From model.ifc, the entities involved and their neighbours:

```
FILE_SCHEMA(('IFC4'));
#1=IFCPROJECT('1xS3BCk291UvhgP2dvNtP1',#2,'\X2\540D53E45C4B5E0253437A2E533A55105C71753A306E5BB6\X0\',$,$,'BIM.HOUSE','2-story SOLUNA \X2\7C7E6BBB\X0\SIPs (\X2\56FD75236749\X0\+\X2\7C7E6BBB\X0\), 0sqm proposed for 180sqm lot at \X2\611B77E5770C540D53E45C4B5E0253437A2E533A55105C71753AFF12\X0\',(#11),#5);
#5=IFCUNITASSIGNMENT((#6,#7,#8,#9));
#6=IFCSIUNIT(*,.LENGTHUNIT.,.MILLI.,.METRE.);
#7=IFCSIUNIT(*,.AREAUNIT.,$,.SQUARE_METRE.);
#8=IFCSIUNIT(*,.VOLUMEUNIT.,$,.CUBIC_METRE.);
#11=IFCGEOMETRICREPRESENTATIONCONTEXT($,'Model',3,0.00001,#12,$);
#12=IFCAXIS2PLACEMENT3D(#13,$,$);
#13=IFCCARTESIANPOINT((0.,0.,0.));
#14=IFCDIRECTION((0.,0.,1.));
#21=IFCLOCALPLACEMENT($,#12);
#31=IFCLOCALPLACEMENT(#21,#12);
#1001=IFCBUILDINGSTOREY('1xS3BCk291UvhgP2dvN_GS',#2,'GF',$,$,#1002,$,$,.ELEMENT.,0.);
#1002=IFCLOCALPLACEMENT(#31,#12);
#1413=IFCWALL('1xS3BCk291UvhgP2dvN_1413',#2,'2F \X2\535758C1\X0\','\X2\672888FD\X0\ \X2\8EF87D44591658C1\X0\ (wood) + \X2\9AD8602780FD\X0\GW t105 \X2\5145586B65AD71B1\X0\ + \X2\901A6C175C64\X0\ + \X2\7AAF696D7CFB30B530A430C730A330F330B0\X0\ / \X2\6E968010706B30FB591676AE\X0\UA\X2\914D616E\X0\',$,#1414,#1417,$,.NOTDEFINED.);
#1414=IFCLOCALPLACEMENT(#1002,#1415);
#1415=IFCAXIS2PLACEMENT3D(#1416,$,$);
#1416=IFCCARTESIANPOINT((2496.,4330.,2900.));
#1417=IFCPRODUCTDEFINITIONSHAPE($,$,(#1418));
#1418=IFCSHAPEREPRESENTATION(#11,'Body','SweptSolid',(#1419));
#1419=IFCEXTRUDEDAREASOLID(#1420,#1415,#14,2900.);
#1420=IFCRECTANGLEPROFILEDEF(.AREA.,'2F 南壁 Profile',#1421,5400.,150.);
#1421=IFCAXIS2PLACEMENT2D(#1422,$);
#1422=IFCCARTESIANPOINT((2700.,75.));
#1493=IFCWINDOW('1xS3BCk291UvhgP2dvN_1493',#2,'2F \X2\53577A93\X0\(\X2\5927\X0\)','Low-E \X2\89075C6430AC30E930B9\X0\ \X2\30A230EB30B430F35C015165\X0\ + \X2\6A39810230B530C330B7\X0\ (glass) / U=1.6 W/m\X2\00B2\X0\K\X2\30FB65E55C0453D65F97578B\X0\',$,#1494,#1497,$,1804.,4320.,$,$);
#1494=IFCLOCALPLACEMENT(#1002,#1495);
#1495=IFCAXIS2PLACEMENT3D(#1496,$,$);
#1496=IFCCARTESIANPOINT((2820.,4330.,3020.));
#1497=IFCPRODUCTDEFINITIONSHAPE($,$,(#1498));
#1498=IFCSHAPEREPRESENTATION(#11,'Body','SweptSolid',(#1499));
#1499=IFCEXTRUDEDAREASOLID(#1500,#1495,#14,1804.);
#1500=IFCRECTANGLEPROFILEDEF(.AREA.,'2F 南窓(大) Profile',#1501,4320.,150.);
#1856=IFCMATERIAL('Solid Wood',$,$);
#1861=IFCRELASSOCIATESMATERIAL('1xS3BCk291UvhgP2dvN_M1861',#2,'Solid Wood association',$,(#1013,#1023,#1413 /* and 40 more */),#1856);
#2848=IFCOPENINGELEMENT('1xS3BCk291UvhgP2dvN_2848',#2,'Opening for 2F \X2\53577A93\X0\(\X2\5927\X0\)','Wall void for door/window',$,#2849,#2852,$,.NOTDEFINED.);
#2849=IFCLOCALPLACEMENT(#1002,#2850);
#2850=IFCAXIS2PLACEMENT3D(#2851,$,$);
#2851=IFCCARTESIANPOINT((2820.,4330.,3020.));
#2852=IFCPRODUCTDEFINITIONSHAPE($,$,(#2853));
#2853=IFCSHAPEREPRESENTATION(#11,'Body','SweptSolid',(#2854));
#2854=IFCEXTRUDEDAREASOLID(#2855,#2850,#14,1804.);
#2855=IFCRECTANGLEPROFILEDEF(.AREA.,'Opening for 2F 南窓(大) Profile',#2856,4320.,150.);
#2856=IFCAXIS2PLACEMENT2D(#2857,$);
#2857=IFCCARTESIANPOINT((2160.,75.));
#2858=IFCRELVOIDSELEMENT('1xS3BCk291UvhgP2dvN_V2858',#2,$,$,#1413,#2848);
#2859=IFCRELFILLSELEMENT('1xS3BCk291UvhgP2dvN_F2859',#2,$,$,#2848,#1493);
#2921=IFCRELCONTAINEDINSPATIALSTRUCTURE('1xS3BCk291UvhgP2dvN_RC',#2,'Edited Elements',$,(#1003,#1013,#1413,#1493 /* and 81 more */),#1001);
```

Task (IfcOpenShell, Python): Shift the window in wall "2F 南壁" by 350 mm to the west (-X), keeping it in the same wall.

```python
import ifcopenshell
import ifcopenshell.api.geometry
import ifcopenshell.util.placement
import ifcopenshell.util.unit

model = ifcopenshell.open("model.ifc")
unit_scale = ifcopenshell.util.unit.calculate_unit_scale(model)

window = model.by_guid("1xS3BCk291UvhgP2dvN_1493")
opening = window.FillsVoids[0].RelatingOpeningElement
wall = opening.VoidsElements[0].RelatingBuildingElement

wall_matrix = ifcopenshell.util.placement.get_local_placement(wall.ObjectPlacement)
shift = wall_matrix[:3, 0] * -0.35 / unit_scale
before = ifcopenshell.util.placement.get_local_placement(window.ObjectPlacement)[:3, 3].copy()

# The window is not placed relative to its opening, so move both.
for product in (opening, window):
    matrix = ifcopenshell.util.placement.get_local_placement(product.ObjectPlacement)
    matrix[:3, 3] += shift
    ifcopenshell.api.geometry.edit_object_placement(model, product=product, matrix=matrix, is_si=False)

after = ifcopenshell.util.placement.get_local_placement(window.ObjectPlacement)[:3, 3]
print("window moved by", (after - before).round(3) + 0.0)

model.write("model-out.ifc")
```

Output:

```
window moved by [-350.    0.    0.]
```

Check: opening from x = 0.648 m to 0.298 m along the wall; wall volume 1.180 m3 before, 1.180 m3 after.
